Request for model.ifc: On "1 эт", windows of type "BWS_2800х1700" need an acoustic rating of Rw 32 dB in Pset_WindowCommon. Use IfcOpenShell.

First a look at what the model holds.

```python
import ifcopenshell
import ifcopenshell.util.element

model = ifcopenshell.open("model.ifc")
print(model.schema)
storey = next(s for s in model.by_type("IfcBuildingStorey") if s.Name == "1 эт")
windows = [e for e in ifcopenshell.util.element.get_decomposition(storey) if e.is_a("IfcWindow")]
seen = {}
for e in windows:
    element_type = ifcopenshell.util.element.get_type(e)
    key = (element_type.Name if element_type != e and element_type else None, ifcopenshell.util.element.get_pset(e, "Pset_WindowCommon", "AcousticRating"))
    seen[key] = seen.get(key, 0) + 1
for (name, value), count in sorted(seen.items(), key=str):
    print(count, "x", name, "|", value)
```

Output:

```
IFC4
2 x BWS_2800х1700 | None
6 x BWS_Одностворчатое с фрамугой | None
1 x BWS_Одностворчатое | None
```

```python
import ifcopenshell
import ifcopenshell.api.pset
import ifcopenshell.util.element

model = ifcopenshell.open("model.ifc")

storey = next(s for s in model.by_type("IfcBuildingStorey") if s.Name == "1 эт")
windows = [e for e in ifcopenshell.util.element.get_decomposition(storey) if e.is_a("IfcWindow")]

count = 0
for e in windows:
    element_type = ifcopenshell.util.element.get_type(e)
    if element_type in (None, e) or element_type.Name != "BWS_2800х1700":
        continue
    # add_pset returns the element's existing set when there is one.
    pset = ifcopenshell.api.pset.add_pset(model, product=e, name="Pset_WindowCommon")
    ifcopenshell.api.pset.edit_pset(model, pset=pset, properties={"AcousticRating": "Rw 32 dB"})
    count += 1

print(count, "windows updated")

model.write("model-out.ifc")
```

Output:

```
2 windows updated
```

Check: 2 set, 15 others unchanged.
